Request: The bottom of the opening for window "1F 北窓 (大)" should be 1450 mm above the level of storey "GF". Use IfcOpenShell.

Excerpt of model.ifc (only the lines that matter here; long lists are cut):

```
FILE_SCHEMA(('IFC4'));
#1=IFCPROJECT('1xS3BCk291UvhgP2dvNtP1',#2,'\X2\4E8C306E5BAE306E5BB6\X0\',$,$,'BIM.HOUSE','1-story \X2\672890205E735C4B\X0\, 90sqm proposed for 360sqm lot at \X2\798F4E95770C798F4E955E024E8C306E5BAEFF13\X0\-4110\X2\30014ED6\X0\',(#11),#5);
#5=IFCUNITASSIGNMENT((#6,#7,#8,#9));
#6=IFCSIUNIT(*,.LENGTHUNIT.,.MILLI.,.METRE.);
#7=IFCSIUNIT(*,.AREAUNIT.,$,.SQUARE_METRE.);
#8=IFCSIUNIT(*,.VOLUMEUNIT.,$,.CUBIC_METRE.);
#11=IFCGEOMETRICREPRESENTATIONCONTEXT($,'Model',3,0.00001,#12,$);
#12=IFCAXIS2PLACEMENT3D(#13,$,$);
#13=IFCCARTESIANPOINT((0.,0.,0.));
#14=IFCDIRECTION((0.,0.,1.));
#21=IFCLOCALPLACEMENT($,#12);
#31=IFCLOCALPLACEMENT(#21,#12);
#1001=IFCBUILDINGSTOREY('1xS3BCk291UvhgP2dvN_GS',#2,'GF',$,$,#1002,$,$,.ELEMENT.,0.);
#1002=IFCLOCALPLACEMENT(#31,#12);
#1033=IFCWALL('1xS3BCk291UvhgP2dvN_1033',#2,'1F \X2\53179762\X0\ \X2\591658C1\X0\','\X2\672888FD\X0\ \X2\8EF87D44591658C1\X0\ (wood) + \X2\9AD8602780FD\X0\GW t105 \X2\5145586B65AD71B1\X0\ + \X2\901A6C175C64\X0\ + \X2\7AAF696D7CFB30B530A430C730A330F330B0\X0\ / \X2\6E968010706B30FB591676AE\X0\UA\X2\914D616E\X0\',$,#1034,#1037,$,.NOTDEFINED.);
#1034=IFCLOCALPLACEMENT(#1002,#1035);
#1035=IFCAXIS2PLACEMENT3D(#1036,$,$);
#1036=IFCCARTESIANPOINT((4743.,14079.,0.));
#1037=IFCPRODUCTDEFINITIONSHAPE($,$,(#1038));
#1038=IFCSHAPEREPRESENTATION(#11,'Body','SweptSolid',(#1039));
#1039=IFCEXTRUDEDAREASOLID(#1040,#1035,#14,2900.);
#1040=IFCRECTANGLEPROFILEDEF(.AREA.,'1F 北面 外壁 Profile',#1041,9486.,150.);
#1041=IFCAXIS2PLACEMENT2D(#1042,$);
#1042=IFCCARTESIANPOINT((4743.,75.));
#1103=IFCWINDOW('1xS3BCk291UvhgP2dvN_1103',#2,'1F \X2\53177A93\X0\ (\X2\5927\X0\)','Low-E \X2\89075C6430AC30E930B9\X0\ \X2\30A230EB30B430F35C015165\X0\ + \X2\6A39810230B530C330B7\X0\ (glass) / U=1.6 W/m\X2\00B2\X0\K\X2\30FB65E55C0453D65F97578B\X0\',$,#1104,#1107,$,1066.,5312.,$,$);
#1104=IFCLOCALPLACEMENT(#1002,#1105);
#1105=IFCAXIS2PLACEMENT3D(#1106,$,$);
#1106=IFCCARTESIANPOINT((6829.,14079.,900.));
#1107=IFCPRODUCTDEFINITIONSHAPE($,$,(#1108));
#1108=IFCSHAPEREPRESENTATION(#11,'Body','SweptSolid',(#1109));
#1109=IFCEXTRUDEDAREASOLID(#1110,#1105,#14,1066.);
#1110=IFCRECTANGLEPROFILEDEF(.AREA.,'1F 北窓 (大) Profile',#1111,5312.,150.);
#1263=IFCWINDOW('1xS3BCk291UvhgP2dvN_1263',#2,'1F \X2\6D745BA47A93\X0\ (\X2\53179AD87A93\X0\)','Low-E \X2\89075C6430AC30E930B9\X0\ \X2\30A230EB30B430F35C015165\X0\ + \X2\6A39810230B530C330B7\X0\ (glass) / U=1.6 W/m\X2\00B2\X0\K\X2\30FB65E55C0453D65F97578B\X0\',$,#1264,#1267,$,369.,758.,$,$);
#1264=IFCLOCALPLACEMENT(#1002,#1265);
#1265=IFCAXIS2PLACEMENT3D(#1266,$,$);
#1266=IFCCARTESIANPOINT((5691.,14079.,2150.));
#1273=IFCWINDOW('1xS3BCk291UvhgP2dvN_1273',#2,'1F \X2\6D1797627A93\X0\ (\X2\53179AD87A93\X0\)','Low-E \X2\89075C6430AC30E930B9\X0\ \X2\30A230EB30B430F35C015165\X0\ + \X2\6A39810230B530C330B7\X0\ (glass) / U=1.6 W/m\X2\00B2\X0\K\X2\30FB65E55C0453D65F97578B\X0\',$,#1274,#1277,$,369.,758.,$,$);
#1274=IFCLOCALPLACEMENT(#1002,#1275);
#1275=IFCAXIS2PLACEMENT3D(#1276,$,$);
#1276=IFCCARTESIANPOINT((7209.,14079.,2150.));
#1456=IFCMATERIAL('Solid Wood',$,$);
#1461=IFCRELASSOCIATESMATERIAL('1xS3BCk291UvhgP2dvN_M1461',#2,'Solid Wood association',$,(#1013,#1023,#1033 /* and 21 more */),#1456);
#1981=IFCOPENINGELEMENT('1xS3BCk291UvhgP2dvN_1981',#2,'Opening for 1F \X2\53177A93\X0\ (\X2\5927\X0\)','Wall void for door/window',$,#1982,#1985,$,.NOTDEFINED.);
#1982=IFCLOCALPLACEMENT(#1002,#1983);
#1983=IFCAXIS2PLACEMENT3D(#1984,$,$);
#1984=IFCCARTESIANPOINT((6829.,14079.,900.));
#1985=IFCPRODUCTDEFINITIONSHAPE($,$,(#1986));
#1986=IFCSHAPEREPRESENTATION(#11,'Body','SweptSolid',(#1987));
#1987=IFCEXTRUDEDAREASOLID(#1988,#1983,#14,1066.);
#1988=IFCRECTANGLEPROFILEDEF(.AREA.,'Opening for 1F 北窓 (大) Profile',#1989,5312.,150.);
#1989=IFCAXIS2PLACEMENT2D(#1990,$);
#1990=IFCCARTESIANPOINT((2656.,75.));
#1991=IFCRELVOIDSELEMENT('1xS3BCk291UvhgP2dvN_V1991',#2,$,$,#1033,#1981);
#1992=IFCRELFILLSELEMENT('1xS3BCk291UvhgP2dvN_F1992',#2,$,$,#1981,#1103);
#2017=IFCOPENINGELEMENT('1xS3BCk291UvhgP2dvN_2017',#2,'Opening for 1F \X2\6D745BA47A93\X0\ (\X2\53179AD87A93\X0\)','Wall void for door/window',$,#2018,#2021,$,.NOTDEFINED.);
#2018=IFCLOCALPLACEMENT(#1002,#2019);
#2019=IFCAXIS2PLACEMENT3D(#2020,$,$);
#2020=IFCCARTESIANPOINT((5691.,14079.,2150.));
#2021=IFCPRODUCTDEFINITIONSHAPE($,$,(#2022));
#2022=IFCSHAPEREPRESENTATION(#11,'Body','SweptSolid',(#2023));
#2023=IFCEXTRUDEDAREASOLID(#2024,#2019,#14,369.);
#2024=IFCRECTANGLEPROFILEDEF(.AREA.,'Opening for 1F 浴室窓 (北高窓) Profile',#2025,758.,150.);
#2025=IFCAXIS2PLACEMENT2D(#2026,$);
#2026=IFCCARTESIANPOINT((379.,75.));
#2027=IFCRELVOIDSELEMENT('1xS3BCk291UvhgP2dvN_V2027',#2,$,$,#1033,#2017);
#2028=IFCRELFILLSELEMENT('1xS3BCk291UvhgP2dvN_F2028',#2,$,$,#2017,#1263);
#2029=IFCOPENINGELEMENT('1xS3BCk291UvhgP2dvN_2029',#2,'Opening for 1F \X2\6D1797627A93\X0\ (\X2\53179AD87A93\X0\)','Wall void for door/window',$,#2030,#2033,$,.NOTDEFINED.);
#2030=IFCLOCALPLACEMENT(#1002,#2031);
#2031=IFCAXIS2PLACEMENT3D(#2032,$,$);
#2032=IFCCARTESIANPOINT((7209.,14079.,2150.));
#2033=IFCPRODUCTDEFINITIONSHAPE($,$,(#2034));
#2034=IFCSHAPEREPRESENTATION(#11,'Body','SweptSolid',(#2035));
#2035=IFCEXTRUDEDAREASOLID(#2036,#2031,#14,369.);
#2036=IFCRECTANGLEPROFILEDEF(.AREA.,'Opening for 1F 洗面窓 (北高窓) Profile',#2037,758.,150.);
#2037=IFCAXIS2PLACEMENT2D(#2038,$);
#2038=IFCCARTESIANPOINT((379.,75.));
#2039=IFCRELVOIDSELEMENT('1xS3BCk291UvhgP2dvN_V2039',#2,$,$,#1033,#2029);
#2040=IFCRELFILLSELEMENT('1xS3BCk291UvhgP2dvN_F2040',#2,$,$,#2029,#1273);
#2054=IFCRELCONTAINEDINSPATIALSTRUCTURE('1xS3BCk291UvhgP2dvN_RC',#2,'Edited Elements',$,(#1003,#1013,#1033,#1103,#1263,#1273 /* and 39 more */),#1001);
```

```python
import numpy as np
import ifcopenshell
import ifcopenshell.api.geometry
import ifcopenshell.geom
import ifcopenshell.util.element
import ifcopenshell.util.placement
import ifcopenshell.util.shape
import ifcopenshell.util.unit

model = ifcopenshell.open("model.ifc")
unit_scale = ifcopenshell.util.unit.calculate_unit_scale(model)

window = model.by_guid("1xS3BCk291UvhgP2dvN_1103")
opening = window.FillsVoids[0].RelatingOpeningElement
storey = ifcopenshell.util.element.get_container(window, ifc_class="IfcBuildingStorey")
level = ifcopenshell.util.placement.get_local_placement(storey.ObjectPlacement)[2, 3]

# The opening's origin need not be at the sill, so measure its lowest point.
shape = ifcopenshell.geom.create_shape(ifcopenshell.geom.settings(), opening)
bottom = ifcopenshell.util.shape.get_shape_bottom_elevation(shape, shape.geometry) / unit_scale
dz = level + 1450.0 - bottom

shift = np.array([0.0, 0.0, dz])
# The window is not placed relative to its opening, so move both.
for product in (opening, window):
    matrix = ifcopenshell.util.placement.get_local_placement(product.ObjectPlacement)
    matrix[:3, 3] += shift
    ifcopenshell.api.geometry.edit_object_placement(model, product=product, matrix=matrix, is_si=False)

print(f"moved by {dz * unit_scale:+.3f} m")

model.write("model_rev.ifc")
```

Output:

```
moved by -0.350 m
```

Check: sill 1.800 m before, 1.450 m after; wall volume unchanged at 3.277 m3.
